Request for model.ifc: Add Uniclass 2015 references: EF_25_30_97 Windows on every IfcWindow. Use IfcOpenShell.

First a look at what the model holds.

```python
import ifcopenshell

model = ifcopenshell.open("model.ifc")
print(model.schema)
print("classifications:", [c.Name for c in model.by_type("IfcClassification")])
for ifc_class in ("IfcDoor", "IfcRoof", "IfcStair", "IfcWall", "IfcWindow"):
    print(ifc_class, len(model.by_type(ifc_class)))
```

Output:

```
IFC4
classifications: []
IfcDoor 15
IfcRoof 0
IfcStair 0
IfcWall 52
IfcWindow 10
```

```python
import ifcopenshell
import ifcopenshell.api.classification

model = ifcopenshell.open("model.ifc")

system = ifcopenshell.api.classification.add_classification(model, classification="Uniclass 2015")

codes = {
    "IfcWindow": ("EF_25_30_97", "Windows"),
}
for ifc_class, (code, name) in codes.items():
    products = model.by_type(ifc_class)
    ifcopenshell.api.classification.add_reference(
        model, products=products, classification=system, identification=code, name=name
    )
    print(code, len(products))

model.write("model_rev.ifc")
```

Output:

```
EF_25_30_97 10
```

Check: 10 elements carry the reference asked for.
